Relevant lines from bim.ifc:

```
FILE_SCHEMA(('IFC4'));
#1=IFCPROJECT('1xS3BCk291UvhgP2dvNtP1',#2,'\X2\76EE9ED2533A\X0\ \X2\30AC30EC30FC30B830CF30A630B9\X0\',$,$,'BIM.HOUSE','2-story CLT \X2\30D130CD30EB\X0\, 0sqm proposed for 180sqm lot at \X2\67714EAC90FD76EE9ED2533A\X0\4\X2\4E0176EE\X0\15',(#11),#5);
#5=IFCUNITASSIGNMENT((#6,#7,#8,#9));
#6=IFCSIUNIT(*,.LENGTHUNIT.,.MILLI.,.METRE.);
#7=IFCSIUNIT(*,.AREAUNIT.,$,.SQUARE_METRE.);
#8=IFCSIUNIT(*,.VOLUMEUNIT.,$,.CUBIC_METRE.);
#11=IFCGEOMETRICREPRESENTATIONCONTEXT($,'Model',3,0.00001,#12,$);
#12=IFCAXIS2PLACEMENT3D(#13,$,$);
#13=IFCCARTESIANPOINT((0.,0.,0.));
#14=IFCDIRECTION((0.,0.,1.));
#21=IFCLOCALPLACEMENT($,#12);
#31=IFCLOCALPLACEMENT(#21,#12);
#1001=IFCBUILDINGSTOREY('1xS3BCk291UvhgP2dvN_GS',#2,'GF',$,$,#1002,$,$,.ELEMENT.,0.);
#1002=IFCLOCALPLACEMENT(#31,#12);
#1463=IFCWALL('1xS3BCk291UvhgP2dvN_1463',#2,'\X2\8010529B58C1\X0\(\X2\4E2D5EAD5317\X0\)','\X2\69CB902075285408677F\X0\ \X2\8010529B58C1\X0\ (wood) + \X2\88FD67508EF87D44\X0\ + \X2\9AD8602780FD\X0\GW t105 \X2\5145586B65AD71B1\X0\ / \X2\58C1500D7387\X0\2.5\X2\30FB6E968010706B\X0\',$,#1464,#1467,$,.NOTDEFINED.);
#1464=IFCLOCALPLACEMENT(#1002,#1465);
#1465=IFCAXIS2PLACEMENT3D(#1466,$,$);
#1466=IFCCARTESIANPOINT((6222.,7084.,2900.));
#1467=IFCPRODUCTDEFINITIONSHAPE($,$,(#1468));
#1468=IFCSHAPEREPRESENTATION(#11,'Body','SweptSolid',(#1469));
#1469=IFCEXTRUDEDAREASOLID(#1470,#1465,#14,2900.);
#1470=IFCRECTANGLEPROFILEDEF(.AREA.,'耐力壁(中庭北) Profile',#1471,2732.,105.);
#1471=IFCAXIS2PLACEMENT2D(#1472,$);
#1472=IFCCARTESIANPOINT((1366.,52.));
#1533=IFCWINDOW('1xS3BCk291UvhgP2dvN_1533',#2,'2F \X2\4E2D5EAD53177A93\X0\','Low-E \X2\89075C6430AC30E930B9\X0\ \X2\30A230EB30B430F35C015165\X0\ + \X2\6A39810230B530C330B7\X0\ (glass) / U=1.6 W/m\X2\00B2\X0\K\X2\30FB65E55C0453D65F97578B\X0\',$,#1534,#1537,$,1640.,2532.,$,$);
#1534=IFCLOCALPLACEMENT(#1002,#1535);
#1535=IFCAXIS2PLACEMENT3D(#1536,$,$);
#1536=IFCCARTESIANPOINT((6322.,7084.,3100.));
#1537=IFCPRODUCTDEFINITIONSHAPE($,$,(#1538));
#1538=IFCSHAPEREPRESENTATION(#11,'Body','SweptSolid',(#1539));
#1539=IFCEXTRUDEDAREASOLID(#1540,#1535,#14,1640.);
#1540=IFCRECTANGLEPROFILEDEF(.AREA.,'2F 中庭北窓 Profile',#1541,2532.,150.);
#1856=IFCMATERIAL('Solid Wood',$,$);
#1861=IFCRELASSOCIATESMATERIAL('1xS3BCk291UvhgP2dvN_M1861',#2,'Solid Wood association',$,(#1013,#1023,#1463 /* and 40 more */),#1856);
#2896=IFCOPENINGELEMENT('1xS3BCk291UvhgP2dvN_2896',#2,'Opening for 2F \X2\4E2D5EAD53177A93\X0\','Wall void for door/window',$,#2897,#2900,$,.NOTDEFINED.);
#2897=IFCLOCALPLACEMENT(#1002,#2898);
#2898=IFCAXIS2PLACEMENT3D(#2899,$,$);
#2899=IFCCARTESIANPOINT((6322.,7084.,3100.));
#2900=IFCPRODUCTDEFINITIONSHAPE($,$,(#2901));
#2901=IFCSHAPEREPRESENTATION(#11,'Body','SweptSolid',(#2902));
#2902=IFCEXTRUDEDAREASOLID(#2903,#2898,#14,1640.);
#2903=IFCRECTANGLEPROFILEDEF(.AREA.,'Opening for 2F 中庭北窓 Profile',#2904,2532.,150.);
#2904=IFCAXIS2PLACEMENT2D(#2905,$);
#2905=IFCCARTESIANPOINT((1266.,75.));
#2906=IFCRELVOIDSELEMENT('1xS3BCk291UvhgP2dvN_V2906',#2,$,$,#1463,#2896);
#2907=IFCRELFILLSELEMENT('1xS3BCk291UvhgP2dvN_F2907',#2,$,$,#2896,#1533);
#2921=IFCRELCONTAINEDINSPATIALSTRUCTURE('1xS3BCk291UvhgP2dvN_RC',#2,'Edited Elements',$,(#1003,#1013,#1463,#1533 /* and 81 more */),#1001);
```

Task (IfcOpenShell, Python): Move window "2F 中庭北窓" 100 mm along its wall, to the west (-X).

```python
import ifcopenshell
import ifcopenshell.api.geometry
import ifcopenshell.util.placement
import ifcopenshell.util.unit

model = ifcopenshell.open("bim.ifc")
unit_scale = ifcopenshell.util.unit.calculate_unit_scale(model)

window = model.by_guid("1xS3BCk291UvhgP2dvN_1533")
opening = window.FillsVoids[0].RelatingOpeningElement
wall = opening.VoidsElements[0].RelatingBuildingElement

wall_matrix = ifcopenshell.util.placement.get_local_placement(wall.ObjectPlacement)
shift = wall_matrix[:3, 0] * -0.1 / unit_scale
before = ifcopenshell.util.placement.get_local_placement(window.ObjectPlacement)[:3, 3].copy()

# The window is not placed relative to its opening, so move both.
for product in (opening, window):
    matrix = ifcopenshell.util.placement.get_local_placement(product.ObjectPlacement)
    matrix[:3, 3] += shift
    ifcopenshell.api.geometry.edit_object_placement(model, product=product, matrix=matrix, is_si=False)

after = ifcopenshell.util.placement.get_local_placement(window.ObjectPlacement)[:3, 3]
print("window moved by", (after - before).round(3) + 0.0)

model.write("bim_rev.ifc")
```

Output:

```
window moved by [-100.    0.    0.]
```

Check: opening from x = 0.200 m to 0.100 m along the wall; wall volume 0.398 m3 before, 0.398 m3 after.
